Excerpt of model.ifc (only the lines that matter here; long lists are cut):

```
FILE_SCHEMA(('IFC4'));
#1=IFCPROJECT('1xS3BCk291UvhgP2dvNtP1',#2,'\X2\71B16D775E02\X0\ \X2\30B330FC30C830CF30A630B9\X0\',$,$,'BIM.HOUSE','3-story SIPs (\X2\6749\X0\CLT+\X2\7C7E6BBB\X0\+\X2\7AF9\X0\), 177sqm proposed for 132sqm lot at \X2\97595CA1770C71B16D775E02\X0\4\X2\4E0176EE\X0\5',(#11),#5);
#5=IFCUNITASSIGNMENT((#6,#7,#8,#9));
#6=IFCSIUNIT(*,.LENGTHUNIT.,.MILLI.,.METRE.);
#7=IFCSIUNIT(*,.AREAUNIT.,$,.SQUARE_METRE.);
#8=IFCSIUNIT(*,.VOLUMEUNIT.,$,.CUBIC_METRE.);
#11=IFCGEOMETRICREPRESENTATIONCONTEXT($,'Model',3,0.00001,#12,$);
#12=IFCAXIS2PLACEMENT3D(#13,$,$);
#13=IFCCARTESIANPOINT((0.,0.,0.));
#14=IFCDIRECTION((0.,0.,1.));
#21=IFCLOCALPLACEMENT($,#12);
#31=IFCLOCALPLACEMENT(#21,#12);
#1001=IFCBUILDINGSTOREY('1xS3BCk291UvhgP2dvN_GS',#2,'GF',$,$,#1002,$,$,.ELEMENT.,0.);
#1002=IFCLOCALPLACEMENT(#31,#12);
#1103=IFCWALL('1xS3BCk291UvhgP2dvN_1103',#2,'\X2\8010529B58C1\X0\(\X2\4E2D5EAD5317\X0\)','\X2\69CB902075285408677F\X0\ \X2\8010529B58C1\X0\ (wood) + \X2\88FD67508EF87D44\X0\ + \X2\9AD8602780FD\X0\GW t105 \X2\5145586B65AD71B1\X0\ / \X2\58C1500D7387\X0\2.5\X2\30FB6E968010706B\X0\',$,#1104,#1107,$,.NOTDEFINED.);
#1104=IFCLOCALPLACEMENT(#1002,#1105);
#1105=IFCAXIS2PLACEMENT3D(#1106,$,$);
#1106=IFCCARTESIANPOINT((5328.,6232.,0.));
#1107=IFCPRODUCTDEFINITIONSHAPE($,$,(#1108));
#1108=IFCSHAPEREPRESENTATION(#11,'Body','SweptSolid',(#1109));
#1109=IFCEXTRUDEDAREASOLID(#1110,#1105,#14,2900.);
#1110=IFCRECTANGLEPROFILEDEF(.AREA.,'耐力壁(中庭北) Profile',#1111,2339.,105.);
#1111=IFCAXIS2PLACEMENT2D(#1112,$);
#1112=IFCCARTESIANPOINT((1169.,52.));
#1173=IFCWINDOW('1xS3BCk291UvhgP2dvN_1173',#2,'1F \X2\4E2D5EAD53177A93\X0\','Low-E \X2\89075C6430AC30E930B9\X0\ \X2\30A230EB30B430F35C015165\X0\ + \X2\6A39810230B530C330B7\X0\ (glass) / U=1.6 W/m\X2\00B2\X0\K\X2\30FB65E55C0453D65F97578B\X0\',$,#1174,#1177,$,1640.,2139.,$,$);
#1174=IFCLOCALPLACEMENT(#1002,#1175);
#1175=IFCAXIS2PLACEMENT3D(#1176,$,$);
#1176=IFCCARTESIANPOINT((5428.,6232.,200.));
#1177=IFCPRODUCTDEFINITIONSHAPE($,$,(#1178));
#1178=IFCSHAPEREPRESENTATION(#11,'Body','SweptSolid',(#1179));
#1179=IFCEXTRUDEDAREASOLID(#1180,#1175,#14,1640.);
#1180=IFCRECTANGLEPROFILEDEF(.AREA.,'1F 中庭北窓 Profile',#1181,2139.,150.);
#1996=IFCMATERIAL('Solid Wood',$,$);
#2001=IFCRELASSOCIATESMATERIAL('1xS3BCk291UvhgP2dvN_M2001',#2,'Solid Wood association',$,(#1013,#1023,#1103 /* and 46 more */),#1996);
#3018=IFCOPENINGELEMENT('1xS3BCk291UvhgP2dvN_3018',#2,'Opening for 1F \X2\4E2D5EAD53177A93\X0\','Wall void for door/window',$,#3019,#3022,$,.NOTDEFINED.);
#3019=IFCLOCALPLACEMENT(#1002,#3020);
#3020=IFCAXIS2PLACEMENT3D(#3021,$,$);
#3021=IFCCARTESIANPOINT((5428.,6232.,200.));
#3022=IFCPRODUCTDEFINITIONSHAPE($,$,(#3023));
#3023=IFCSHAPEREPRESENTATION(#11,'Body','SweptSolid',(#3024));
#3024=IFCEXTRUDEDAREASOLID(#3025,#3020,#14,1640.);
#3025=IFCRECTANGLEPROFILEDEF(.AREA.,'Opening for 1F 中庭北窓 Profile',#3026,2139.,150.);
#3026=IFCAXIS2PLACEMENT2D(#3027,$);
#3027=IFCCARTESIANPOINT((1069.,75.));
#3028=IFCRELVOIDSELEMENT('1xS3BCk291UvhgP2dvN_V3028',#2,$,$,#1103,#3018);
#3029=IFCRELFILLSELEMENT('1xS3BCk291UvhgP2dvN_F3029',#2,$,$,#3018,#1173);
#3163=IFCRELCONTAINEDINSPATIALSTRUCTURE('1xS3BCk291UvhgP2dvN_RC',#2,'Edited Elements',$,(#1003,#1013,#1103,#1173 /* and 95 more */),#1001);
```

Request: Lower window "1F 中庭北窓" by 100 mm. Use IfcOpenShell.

```python
import numpy as np
import ifcopenshell
import ifcopenshell.api.geometry
import ifcopenshell.util.placement
import ifcopenshell.util.unit

model = ifcopenshell.open("model.ifc")
unit_scale = ifcopenshell.util.unit.calculate_unit_scale(model)

window = model.by_guid("1xS3BCk291UvhgP2dvN_1173")
opening = window.FillsVoids[0].RelatingOpeningElement
dz = -0.1 / unit_scale

shift = np.array([0.0, 0.0, dz])
# The window is not placed relative to its opening, so move both.
for product in (opening, window):
    matrix = ifcopenshell.util.placement.get_local_placement(product.ObjectPlacement)
    matrix[:3, 3] += shift
    ifcopenshell.api.geometry.edit_object_placement(model, product=product, matrix=matrix, is_si=False)

print(f"moved by {dz * unit_scale:+.3f} m")

model.write("model_edited.ifc")
```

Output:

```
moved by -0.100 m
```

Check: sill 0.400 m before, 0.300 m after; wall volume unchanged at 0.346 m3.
